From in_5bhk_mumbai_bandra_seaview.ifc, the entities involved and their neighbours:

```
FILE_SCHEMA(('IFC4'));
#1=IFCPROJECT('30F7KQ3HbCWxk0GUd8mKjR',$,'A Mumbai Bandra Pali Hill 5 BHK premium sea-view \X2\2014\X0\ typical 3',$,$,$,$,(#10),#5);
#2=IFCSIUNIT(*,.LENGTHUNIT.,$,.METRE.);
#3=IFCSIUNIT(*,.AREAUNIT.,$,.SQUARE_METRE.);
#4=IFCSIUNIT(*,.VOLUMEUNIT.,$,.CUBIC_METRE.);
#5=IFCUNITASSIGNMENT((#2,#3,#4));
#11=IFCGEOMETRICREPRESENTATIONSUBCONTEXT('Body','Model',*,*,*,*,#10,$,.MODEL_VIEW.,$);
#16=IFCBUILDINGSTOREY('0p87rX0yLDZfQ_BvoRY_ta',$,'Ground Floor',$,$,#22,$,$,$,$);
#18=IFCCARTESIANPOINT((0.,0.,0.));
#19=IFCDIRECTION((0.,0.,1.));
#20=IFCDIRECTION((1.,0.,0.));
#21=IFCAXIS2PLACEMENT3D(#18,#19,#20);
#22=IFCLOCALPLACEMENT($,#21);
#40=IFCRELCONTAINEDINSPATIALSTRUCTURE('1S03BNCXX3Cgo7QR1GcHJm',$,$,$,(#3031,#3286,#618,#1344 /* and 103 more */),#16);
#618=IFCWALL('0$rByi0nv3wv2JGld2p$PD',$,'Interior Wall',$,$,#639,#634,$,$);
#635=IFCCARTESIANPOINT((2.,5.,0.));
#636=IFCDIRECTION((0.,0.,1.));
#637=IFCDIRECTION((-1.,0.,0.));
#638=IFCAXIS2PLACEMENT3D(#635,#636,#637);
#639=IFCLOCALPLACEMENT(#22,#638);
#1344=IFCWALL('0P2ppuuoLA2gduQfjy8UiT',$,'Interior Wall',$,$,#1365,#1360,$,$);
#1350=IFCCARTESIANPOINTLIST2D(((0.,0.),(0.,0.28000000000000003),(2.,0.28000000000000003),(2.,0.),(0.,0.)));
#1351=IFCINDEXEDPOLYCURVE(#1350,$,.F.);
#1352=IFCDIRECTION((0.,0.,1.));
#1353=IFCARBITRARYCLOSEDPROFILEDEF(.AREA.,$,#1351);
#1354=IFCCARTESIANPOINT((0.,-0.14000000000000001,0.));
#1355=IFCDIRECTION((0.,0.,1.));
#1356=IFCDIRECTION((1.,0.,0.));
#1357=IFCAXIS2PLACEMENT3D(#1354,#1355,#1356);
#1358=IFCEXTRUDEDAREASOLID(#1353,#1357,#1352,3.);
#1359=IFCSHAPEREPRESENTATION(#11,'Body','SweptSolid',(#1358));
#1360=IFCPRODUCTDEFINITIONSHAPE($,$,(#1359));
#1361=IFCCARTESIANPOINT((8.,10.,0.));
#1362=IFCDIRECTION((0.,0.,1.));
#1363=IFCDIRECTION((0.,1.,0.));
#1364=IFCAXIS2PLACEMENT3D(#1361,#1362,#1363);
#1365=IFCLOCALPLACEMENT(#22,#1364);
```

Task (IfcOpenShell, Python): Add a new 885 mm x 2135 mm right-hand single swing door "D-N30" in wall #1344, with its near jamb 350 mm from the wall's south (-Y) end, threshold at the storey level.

```python
import numpy as np
import ifcopenshell
import ifcopenshell.api.feature
import ifcopenshell.api.geometry
import ifcopenshell.api.root
import ifcopenshell.api.spatial
import ifcopenshell.geom
import ifcopenshell.util.element
import ifcopenshell.util.placement
import ifcopenshell.util.representation
import ifcopenshell.util.shape
import ifcopenshell.util.unit

model = ifcopenshell.open("in_5bhk_mumbai_bandra_seaview.ifc")
unit_scale = ifcopenshell.util.unit.calculate_unit_scale(model)
settings = ifcopenshell.geom.settings()


def volume(element):
    """Net volume in cubic metres, openings subtracted."""
    shape = ifcopenshell.geom.create_shape(settings, element)
    return ifcopenshell.util.shape.get_volume(shape.geometry)


wall = model.by_guid("0P2ppuuoLA2gduQfjy8UiT")
storey = ifcopenshell.util.element.get_container(wall, ifc_class="IfcBuildingStorey")
context = ifcopenshell.util.representation.get_context(model, "Model", "Body", "MODEL_VIEW")
before = volume(wall)

width, height, from_end, sill = 0.885, 2.135, 0.35, 0.0  # metres

# The wall runs along its own X axis, and the end named is its -X end.
wall_shape = ifcopenshell.geom.create_shape(settings, wall)
x, y, z = ifcopenshell.util.shape.get_vertices(wall_shape.geometry).T
start = x.min() + from_end
face, thickness = float(y.min()), float(y.max() - y.min())
wall_matrix = ifcopenshell.util.placement.get_local_placement(wall.ObjectPlacement)
level = ifcopenshell.util.placement.get_local_placement(storey.ObjectPlacement)[2, 3]


def in_wall(x, y):
    """Placement at x, y metres in the wall's axes, at sill height."""
    matrix = wall_matrix.copy()
    matrix[:, 3] = wall_matrix @ np.array([x / unit_scale, y / unit_scale, 0.0, 1.0])
    matrix[2, 3] = level + sill / unit_scale
    return matrix


# Opening: a box that overshoots both wall faces by 50 mm.
opening = ifcopenshell.api.root.create_entity(model, ifc_class="IfcOpeningElement", predefined_type="OPENING")
box = ifcopenshell.api.geometry.add_wall_representation(
    model, context=context, length=width, height=height, thickness=thickness + 0.1
)
ifcopenshell.api.geometry.assign_representation(model, product=opening, representation=box)
ifcopenshell.api.geometry.edit_object_placement(model, product=opening, matrix=in_wall(start, face - 0.05), is_si=False)
ifcopenshell.api.feature.add_feature(model, feature=opening, element=wall)

door = ifcopenshell.api.root.create_entity(model, ifc_class="IfcDoor", name="D-N30", predefined_type="DOOR")
door.OverallWidth, door.OverallHeight = width / unit_scale, height / unit_scale
door.OperationType = "SINGLE_SWING_RIGHT"
body = ifcopenshell.api.geometry.add_door_representation(
    model,
    context=context,
    overall_width=door.OverallWidth,
    overall_height=door.OverallHeight,
    operation_type="SINGLE_SWING_RIGHT",
    lining_properties={"LiningDepth": thickness / unit_scale, "ThresholdDepth": thickness / unit_scale},
)
ifcopenshell.api.geometry.assign_representation(model, product=door, representation=body)
ifcopenshell.api.spatial.assign_container(model, products=[door], relating_structure=storey)
ifcopenshell.api.feature.add_filling(model, opening=opening, element=door)

# The lining spans the wall, so the door starts at the wall face.
ifcopenshell.api.geometry.edit_object_placement(model, product=door, matrix=in_wall(start, face), is_si=False)

after = volume(wall)

print(f"wall volume {before:.3f} -> {after:.3f} m3")

model.write("in_5bhk_mumbai_bandra_seaview_edited.ifc")
```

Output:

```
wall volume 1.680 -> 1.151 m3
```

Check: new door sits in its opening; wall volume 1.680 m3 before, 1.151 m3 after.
